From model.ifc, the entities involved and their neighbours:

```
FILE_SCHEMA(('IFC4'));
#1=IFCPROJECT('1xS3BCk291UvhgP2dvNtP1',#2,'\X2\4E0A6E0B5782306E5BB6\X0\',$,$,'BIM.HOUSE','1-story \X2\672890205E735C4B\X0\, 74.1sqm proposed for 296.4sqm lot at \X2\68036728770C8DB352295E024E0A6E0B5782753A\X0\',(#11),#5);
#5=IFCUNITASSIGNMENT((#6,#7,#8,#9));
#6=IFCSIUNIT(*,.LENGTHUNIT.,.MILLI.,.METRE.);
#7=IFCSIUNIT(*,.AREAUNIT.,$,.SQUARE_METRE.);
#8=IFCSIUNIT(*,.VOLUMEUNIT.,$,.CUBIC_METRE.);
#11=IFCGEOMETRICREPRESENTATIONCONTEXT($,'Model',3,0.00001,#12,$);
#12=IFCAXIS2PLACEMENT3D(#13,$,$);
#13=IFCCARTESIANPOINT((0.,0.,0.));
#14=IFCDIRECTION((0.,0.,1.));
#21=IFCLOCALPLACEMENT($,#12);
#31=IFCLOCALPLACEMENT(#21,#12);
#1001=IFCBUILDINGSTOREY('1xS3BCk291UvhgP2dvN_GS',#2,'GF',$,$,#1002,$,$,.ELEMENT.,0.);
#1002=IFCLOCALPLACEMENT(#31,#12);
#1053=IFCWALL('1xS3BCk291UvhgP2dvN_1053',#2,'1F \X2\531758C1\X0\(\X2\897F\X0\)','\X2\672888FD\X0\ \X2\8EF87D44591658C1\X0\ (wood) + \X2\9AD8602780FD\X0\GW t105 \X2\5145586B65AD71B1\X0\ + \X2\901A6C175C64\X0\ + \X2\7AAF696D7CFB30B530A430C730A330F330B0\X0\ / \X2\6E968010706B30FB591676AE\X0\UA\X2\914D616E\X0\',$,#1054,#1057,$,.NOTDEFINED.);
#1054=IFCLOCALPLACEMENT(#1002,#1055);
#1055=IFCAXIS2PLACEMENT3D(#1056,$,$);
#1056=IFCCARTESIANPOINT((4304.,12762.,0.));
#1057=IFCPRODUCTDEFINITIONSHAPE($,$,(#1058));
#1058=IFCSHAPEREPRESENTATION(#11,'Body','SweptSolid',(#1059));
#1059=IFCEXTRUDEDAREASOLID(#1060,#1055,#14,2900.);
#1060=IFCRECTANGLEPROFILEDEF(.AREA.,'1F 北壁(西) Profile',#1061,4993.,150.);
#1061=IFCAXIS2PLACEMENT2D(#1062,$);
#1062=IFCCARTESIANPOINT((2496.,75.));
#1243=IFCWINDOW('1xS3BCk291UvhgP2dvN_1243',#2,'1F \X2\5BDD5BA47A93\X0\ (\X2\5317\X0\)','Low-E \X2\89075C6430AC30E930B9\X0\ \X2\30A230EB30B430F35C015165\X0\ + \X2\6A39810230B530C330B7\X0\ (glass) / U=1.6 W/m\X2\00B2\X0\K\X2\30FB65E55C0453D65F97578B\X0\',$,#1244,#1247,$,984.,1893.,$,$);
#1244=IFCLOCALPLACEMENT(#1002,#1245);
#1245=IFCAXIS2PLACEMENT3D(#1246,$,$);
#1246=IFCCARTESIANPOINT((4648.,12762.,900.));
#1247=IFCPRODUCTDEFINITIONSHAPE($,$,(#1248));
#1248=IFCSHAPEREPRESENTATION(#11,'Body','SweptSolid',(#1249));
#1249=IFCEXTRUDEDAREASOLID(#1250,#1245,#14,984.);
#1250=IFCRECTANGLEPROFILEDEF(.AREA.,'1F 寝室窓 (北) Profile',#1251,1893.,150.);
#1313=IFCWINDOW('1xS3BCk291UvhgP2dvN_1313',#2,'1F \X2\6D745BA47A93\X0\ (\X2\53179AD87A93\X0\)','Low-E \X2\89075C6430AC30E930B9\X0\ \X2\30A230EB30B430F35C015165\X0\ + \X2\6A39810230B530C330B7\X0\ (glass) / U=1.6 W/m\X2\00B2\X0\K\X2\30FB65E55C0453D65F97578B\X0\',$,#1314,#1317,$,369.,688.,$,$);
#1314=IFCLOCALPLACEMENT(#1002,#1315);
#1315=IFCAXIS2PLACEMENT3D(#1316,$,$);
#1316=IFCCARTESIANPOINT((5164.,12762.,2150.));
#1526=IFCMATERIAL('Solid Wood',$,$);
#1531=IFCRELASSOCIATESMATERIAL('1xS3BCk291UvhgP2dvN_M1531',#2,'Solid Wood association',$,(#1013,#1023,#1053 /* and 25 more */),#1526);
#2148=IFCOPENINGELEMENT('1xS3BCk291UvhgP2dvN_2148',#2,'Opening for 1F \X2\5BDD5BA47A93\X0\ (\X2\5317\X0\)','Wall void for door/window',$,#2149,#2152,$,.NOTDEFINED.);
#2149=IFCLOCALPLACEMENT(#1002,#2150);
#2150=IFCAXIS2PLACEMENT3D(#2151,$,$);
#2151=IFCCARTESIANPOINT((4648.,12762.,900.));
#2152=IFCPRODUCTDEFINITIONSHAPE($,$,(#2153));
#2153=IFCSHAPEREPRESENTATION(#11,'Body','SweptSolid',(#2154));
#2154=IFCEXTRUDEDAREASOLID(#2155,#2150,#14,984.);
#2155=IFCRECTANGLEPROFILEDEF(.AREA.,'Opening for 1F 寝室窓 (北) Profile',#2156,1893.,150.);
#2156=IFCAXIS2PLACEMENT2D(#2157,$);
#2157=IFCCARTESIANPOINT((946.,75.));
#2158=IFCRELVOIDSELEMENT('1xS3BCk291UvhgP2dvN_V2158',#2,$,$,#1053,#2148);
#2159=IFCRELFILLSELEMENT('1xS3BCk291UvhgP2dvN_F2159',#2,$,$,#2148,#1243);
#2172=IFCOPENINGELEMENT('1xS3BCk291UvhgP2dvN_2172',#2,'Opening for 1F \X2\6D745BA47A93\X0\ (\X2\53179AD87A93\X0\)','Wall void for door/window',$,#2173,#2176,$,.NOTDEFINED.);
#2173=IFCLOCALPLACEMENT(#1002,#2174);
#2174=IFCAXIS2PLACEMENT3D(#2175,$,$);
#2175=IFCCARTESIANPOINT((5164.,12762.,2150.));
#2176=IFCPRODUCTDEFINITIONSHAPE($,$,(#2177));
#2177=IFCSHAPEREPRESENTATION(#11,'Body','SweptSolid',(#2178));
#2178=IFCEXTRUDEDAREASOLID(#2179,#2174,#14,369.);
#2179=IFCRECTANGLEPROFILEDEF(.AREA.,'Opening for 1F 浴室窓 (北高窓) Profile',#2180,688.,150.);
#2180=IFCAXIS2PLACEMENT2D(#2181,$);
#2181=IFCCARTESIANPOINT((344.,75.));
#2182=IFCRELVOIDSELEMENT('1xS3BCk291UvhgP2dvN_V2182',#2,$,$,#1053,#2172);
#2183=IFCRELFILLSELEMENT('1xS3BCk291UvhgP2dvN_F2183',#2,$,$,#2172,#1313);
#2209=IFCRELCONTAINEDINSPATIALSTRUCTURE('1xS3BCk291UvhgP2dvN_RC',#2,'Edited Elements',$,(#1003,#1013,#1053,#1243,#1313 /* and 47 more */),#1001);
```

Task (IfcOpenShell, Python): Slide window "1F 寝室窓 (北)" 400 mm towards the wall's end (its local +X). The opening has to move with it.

```python
import ifcopenshell
import ifcopenshell.api.geometry
import ifcopenshell.util.placement
import ifcopenshell.util.unit

model = ifcopenshell.open("model.ifc")
unit_scale = ifcopenshell.util.unit.calculate_unit_scale(model)

window = model.by_id(1243)
opening = window.FillsVoids[0].RelatingOpeningElement
wall = opening.VoidsElements[0].RelatingBuildingElement

wall_matrix = ifcopenshell.util.placement.get_local_placement(wall.ObjectPlacement)
shift = wall_matrix[:3, 0] * 0.4 / unit_scale
before = ifcopenshell.util.placement.get_local_placement(window.ObjectPlacement)[:3, 3].copy()

# The window is not placed relative to its opening, so move both.
for product in (opening, window):
    matrix = ifcopenshell.util.placement.get_local_placement(product.ObjectPlacement)
    matrix[:3, 3] += shift
    ifcopenshell.api.geometry.edit_object_placement(model, product=product, matrix=matrix, is_si=False)

after = ifcopenshell.util.placement.get_local_placement(window.ObjectPlacement)[:3, 3]
print("window moved by", (after - before).round(3) + 0.0)

model.write("model_v2.ifc")
```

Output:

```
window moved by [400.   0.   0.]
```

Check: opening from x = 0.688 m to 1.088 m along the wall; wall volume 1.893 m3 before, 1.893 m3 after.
